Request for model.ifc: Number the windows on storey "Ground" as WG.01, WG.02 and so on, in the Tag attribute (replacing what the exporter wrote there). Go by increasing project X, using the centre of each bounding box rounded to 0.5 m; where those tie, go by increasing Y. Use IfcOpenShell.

First a look at what the model holds.

```python
import ifcopenshell
import ifcopenshell.util.element
import ifcopenshell.util.placement

model = ifcopenshell.open("model.ifc")
print(model.schema)
storey = next(s for s in model.by_type("IfcBuildingStorey") if s.Name == "Ground")
windows = [e for e in ifcopenshell.util.element.get_decomposition(storey) if e.is_a("IfcWindow")]
for e in sorted(windows, key=lambda e: e.id()):
    origin = ifcopenshell.util.placement.get_local_placement(e.ObjectPlacement)[:3, 3]
    print(e.id(), e.Tag, e.Name, origin.round(2) + 0.0, sep=" | ")
```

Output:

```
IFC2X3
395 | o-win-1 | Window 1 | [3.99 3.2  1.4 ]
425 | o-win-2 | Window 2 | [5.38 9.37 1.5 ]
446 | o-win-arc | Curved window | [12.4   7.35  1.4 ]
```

```python
import ifcopenshell
import ifcopenshell.geom
import ifcopenshell.util.element
import ifcopenshell.util.shape

model = ifcopenshell.open("model.ifc")
settings = ifcopenshell.geom.settings()
settings.set("use-world-coords", True)


def centre(element):
    shape = ifcopenshell.geom.create_shape(settings, element)
    return ifcopenshell.util.shape.get_bbox_centroid(shape.geometry)


storey = next(s for s in model.by_type("IfcBuildingStorey") if s.Name == "Ground")
windows = [e for e in ifcopenshell.util.element.get_decomposition(storey) if e.is_a("IfcWindow")]

# Insertion points can sit at a corner or the storey origin, so sort by the geometry (in metres).
centres = {e: centre(e) for e in windows}
windows.sort(key=lambda e: (round(centres[e][0] / 0.5), centres[e][1]))

for i, e in enumerate(windows, start=1):
    number = f"WG.{i:02d}"
    e.Tag = number
    print(e.id(), number)

model.write("model_v2.ifc")
```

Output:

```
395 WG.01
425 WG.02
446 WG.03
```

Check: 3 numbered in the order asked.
